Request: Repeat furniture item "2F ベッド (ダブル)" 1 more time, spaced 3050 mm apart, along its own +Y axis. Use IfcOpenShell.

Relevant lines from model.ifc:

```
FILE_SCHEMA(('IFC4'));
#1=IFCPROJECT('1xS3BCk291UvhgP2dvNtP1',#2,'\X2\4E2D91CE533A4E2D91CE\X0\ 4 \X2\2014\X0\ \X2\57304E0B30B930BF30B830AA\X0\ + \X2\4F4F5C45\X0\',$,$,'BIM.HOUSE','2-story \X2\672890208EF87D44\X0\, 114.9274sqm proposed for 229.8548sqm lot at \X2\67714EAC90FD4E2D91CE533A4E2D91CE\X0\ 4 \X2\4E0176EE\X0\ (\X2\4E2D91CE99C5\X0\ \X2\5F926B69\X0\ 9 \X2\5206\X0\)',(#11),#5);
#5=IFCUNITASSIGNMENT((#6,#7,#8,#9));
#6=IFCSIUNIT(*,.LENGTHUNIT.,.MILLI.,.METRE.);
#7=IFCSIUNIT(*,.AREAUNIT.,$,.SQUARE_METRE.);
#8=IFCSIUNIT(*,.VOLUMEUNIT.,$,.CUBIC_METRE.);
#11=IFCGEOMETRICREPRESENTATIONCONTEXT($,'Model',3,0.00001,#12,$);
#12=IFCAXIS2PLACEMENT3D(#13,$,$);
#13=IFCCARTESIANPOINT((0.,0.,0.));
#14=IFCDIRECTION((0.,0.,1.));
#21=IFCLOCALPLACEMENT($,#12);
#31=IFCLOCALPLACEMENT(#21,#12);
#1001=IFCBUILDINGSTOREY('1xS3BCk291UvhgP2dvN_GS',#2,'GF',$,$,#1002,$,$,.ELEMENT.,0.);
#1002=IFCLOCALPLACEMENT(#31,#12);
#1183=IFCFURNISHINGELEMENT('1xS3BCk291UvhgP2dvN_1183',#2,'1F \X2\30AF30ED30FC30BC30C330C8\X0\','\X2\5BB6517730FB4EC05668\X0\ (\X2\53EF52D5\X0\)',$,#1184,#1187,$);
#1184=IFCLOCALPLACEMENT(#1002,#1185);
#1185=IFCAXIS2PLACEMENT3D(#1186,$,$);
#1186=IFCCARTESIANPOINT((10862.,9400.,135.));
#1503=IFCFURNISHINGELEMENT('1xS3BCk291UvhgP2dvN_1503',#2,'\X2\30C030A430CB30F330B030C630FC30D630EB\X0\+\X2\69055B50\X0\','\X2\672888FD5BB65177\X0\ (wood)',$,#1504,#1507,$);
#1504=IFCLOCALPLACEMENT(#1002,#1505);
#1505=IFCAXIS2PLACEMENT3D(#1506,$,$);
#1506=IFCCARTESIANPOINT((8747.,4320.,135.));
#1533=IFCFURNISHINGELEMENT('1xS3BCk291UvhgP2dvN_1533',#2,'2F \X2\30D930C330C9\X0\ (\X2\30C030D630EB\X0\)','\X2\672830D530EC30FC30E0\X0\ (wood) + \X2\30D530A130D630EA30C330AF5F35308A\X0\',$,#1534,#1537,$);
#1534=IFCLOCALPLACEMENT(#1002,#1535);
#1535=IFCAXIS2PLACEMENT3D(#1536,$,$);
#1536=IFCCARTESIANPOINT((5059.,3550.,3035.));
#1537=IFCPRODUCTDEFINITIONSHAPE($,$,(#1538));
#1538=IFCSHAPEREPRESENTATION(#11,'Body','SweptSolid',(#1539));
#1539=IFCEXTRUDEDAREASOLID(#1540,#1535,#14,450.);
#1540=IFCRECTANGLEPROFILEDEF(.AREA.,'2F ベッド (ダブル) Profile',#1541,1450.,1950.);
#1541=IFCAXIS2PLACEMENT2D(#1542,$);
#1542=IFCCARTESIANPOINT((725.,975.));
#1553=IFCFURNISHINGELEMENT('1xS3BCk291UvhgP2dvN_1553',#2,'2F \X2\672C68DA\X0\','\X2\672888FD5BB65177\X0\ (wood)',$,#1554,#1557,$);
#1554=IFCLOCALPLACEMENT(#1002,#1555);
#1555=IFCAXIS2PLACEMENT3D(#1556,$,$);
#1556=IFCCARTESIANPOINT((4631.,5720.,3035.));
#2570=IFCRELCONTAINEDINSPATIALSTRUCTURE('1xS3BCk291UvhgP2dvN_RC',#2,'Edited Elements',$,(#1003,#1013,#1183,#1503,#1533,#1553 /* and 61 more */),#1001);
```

```python
import ifcopenshell
import ifcopenshell.api.geometry
import ifcopenshell.api.root
import ifcopenshell.util.element
import ifcopenshell.util.placement

model = ifcopenshell.open("model.ifc")


def reuse_history(source, copy):
    """copy_class also copies each property set's owner history, people and application; keep the originals."""
    for rel in copy.IsDefinedBy:
        if rel.is_a("IfcRelDefinesByProperties") and (history := rel.RelatingPropertyDefinition.OwnerHistory):
            rel.RelatingPropertyDefinition.OwnerHistory = source.OwnerHistory
            ifcopenshell.util.element.remove_deep2(model, history)


source = model.by_id(1533)
base = ifcopenshell.util.placement.get_local_placement(source.ObjectPlacement)
step = base[:3, 1] * 3050.0

for i in range(1, 2):
    copy = ifcopenshell.api.root.copy_class(model, product=source)
    copy.Representation = ifcopenshell.util.element.copy_deep(
        model, source.Representation, exclude=["IfcGeometricRepresentationContext", "IfcRepresentationMap"]
    )
    reuse_history(source, copy)
    matrix = base.copy()
    matrix[:3, 3] += i * step
    print("added at", matrix[:3, 3].round(3) + 0.0)
    ifcopenshell.api.geometry.edit_object_placement(model, product=copy, matrix=matrix, is_si=False)

model.write("model_updated.ifc")
```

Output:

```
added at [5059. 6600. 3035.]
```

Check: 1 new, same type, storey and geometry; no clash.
